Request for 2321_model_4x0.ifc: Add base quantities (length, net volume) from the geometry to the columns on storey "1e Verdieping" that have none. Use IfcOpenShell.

First a look at what the model holds.

```python
import ifcopenshell
import ifcopenshell.util.element
import ifcopenshell.util.unit

model = ifcopenshell.open("2321_model_4x0.ifc")
print(model.schema)
for unit_type in ("LENGTHUNIT", "AREAUNIT", "VOLUMEUNIT"):
    print(unit_type, ifcopenshell.util.unit.calculate_unit_scale(model, unit_type))
storey = next(s for s in model.by_type("IfcBuildingStorey") if s.Name == "1e Verdieping")
columns = [e for e in ifcopenshell.util.element.get_decomposition(storey) if e.is_a("IfcColumn")]
for e in sorted(columns, key=lambda e: e.id()):
    print(e.id(), e.is_a(), e.Name, list(ifcopenshell.util.element.get_psets(e, qtos_only=True)), sep=" | ")
```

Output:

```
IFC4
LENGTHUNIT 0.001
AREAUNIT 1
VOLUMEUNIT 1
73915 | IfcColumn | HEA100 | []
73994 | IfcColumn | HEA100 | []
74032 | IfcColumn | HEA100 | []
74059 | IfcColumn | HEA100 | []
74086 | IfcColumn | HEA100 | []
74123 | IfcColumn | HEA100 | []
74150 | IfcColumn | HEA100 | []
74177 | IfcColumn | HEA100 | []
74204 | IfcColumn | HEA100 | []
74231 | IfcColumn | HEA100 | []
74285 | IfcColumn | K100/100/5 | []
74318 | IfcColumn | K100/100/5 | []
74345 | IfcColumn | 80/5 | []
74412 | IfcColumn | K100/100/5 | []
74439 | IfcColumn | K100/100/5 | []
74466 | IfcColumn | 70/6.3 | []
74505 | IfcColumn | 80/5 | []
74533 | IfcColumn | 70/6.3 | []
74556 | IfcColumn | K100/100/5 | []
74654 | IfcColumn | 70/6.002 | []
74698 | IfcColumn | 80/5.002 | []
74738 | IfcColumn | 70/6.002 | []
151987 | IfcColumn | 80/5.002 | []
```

```python
import ifcopenshell
import ifcopenshell.api.pset
import ifcopenshell.geom
import ifcopenshell.util.element
import ifcopenshell.util.shape
import ifcopenshell.util.unit

model = ifcopenshell.open("2321_model_4x0.ifc")
unit_scale = ifcopenshell.util.unit.calculate_unit_scale(model)
volume_scale = ifcopenshell.util.unit.calculate_unit_scale(model, "VOLUMEUNIT")
settings = ifcopenshell.geom.settings()

storey = next(s for s in model.by_type("IfcBuildingStorey") if s.Name == "1e Verdieping")
columns = [e for e in ifcopenshell.util.element.get_decomposition(storey) if e.is_a("IfcColumn")]

for e in sorted(columns, key=lambda e: e.id()):
    if ifcopenshell.util.element.get_psets(e, qtos_only=True, should_inherit=False):
        continue
    # Geometry comes back in metres, in the element's own axes.
    shape = ifcopenshell.geom.create_shape(settings, e)
    values = {
        "Length": ifcopenshell.util.shape.get_z(shape.geometry) / unit_scale,
        "NetVolume": ifcopenshell.util.shape.get_volume(shape.geometry) / volume_scale,
    }
    qto = ifcopenshell.api.pset.add_qto(model, product=e, name="Qto_ColumnBaseQuantities")
    ifcopenshell.api.pset.edit_qto(model, qto=qto, properties=values)
    print(e.id(), {k: round(v, 3) for k, v in values.items()})

model.write("2321_model_4x0_updated.ifc")
```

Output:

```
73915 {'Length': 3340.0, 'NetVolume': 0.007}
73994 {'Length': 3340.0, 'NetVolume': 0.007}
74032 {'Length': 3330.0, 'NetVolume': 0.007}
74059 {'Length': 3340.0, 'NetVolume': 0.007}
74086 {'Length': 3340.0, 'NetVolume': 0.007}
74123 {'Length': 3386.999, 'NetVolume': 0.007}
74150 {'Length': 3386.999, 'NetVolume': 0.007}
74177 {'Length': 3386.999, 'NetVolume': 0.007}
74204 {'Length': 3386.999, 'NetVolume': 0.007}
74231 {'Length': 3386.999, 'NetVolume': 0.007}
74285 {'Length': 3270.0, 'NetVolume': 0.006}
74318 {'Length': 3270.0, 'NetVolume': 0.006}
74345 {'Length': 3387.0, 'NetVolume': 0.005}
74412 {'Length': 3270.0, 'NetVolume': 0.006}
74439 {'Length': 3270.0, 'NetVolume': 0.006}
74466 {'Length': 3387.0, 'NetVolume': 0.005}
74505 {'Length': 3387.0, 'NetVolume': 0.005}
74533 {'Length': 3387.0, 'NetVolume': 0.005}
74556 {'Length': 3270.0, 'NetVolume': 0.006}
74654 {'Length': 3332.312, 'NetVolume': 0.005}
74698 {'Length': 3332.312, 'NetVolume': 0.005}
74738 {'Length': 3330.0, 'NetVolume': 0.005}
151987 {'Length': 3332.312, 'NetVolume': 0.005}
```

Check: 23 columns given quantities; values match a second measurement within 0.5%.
